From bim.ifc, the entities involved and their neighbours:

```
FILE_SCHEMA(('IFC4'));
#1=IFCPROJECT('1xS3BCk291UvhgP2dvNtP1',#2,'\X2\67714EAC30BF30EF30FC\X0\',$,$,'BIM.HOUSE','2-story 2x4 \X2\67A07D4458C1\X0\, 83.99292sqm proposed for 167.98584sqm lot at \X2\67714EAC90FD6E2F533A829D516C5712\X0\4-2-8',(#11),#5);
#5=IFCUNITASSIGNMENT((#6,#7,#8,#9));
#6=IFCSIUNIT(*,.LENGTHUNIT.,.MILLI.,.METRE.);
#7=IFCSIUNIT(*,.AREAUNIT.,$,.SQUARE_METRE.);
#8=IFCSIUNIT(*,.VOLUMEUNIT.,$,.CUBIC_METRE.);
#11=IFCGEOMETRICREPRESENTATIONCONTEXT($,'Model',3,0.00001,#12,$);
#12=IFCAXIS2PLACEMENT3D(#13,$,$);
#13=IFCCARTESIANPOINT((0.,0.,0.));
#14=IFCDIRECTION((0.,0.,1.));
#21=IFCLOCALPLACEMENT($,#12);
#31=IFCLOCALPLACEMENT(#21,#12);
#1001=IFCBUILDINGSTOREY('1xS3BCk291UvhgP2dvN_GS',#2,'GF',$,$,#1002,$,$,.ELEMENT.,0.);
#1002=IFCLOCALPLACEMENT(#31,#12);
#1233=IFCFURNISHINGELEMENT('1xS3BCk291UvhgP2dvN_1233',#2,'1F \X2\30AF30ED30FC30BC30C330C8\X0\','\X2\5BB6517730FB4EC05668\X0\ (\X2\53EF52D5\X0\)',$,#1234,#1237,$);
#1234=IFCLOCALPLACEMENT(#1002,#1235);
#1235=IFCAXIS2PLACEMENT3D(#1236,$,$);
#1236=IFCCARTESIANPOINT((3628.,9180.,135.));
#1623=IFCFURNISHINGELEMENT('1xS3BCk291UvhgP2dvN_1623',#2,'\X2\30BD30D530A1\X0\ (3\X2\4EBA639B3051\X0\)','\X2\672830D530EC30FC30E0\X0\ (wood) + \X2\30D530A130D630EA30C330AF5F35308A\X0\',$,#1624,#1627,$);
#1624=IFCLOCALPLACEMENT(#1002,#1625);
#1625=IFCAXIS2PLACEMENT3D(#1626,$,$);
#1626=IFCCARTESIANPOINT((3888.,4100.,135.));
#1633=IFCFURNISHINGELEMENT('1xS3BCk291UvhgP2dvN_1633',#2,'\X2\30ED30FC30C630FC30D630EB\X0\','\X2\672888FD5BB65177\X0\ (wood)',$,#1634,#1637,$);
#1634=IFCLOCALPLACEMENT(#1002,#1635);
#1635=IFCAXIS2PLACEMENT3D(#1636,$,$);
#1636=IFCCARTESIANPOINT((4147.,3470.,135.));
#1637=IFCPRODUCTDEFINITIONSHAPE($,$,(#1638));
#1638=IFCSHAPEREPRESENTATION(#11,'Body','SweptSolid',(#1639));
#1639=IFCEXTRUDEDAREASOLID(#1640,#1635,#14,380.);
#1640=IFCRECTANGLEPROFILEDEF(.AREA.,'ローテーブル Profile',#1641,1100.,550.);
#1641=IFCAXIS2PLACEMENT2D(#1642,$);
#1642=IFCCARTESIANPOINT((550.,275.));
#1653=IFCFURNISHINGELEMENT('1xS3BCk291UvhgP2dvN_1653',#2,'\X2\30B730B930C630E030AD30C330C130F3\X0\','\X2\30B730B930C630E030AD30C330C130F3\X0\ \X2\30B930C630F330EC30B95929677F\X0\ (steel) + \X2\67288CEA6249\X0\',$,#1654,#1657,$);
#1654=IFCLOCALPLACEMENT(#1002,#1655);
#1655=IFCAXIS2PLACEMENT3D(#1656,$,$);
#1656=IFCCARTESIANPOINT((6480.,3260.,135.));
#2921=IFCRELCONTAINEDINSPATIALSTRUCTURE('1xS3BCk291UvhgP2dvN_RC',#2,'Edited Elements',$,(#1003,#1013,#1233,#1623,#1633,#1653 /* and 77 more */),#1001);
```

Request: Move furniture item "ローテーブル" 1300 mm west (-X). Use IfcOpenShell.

```python
import ifcopenshell
import ifcopenshell.api.geometry
import ifcopenshell.util.placement

model = ifcopenshell.open("bim.ifc")

item = model.by_guid("1xS3BCk291UvhgP2dvN_1633")
matrix = ifcopenshell.util.placement.get_local_placement(item.ObjectPlacement)
matrix[0, 3] -= 1300.0
ifcopenshell.api.geometry.edit_object_placement(model, product=item, matrix=matrix, is_si=False)

print(ifcopenshell.util.placement.get_local_placement(item.ObjectPlacement).round(3) + 0.0)

model.write("bim_rev.ifc")
```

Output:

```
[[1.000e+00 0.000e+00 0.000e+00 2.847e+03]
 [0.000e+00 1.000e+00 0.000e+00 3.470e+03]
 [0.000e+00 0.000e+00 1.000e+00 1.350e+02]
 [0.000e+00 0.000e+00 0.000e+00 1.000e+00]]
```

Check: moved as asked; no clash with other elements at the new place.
